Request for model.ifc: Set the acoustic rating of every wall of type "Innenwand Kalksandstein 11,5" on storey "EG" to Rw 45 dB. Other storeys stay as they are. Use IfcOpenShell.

First a look at what the model holds.

```python
import ifcopenshell
import ifcopenshell.util.element

model = ifcopenshell.open("model.ifc")
print(model.schema)
storey = next(s for s in model.by_type("IfcBuildingStorey") if s.Name == "EG")
walls = [e for e in ifcopenshell.util.element.get_decomposition(storey) if e.is_a("IfcWall")]
seen = {}
for e in walls:
    element_type = ifcopenshell.util.element.get_type(e)
    key = (element_type.Name if element_type != e and element_type else None, ifcopenshell.util.element.get_pset(e, "Pset_WallCommon", "AcousticRating"))
    seen[key] = seen.get(key, 0) + 1
for (name, value), count in sorted(seen.items(), key=str):
    print(count, "x", name, "|", value)
```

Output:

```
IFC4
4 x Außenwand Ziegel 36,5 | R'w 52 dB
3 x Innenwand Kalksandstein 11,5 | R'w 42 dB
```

```python
import ifcopenshell
import ifcopenshell.api.pset
import ifcopenshell.util.element

model = ifcopenshell.open("model.ifc")

storey = next(s for s in model.by_type("IfcBuildingStorey") if s.Name == "EG")
walls = [e for e in ifcopenshell.util.element.get_decomposition(storey) if e.is_a("IfcWall")]

count = 0
for e in walls:
    element_type = ifcopenshell.util.element.get_type(e)
    if element_type in (None, e) or element_type.Name != "Innenwand Kalksandstein 11,5":
        continue
    # add_pset returns the element's existing set when there is one.
    pset = ifcopenshell.api.pset.add_pset(model, product=e, name="Pset_WallCommon")
    ifcopenshell.api.pset.edit_pset(model, pset=pset, properties={"AcousticRating": "Rw 45 dB"})
    count += 1

print(count, "walls updated")

model.write("model_updated.ifc")
```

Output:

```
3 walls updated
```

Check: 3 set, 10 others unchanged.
